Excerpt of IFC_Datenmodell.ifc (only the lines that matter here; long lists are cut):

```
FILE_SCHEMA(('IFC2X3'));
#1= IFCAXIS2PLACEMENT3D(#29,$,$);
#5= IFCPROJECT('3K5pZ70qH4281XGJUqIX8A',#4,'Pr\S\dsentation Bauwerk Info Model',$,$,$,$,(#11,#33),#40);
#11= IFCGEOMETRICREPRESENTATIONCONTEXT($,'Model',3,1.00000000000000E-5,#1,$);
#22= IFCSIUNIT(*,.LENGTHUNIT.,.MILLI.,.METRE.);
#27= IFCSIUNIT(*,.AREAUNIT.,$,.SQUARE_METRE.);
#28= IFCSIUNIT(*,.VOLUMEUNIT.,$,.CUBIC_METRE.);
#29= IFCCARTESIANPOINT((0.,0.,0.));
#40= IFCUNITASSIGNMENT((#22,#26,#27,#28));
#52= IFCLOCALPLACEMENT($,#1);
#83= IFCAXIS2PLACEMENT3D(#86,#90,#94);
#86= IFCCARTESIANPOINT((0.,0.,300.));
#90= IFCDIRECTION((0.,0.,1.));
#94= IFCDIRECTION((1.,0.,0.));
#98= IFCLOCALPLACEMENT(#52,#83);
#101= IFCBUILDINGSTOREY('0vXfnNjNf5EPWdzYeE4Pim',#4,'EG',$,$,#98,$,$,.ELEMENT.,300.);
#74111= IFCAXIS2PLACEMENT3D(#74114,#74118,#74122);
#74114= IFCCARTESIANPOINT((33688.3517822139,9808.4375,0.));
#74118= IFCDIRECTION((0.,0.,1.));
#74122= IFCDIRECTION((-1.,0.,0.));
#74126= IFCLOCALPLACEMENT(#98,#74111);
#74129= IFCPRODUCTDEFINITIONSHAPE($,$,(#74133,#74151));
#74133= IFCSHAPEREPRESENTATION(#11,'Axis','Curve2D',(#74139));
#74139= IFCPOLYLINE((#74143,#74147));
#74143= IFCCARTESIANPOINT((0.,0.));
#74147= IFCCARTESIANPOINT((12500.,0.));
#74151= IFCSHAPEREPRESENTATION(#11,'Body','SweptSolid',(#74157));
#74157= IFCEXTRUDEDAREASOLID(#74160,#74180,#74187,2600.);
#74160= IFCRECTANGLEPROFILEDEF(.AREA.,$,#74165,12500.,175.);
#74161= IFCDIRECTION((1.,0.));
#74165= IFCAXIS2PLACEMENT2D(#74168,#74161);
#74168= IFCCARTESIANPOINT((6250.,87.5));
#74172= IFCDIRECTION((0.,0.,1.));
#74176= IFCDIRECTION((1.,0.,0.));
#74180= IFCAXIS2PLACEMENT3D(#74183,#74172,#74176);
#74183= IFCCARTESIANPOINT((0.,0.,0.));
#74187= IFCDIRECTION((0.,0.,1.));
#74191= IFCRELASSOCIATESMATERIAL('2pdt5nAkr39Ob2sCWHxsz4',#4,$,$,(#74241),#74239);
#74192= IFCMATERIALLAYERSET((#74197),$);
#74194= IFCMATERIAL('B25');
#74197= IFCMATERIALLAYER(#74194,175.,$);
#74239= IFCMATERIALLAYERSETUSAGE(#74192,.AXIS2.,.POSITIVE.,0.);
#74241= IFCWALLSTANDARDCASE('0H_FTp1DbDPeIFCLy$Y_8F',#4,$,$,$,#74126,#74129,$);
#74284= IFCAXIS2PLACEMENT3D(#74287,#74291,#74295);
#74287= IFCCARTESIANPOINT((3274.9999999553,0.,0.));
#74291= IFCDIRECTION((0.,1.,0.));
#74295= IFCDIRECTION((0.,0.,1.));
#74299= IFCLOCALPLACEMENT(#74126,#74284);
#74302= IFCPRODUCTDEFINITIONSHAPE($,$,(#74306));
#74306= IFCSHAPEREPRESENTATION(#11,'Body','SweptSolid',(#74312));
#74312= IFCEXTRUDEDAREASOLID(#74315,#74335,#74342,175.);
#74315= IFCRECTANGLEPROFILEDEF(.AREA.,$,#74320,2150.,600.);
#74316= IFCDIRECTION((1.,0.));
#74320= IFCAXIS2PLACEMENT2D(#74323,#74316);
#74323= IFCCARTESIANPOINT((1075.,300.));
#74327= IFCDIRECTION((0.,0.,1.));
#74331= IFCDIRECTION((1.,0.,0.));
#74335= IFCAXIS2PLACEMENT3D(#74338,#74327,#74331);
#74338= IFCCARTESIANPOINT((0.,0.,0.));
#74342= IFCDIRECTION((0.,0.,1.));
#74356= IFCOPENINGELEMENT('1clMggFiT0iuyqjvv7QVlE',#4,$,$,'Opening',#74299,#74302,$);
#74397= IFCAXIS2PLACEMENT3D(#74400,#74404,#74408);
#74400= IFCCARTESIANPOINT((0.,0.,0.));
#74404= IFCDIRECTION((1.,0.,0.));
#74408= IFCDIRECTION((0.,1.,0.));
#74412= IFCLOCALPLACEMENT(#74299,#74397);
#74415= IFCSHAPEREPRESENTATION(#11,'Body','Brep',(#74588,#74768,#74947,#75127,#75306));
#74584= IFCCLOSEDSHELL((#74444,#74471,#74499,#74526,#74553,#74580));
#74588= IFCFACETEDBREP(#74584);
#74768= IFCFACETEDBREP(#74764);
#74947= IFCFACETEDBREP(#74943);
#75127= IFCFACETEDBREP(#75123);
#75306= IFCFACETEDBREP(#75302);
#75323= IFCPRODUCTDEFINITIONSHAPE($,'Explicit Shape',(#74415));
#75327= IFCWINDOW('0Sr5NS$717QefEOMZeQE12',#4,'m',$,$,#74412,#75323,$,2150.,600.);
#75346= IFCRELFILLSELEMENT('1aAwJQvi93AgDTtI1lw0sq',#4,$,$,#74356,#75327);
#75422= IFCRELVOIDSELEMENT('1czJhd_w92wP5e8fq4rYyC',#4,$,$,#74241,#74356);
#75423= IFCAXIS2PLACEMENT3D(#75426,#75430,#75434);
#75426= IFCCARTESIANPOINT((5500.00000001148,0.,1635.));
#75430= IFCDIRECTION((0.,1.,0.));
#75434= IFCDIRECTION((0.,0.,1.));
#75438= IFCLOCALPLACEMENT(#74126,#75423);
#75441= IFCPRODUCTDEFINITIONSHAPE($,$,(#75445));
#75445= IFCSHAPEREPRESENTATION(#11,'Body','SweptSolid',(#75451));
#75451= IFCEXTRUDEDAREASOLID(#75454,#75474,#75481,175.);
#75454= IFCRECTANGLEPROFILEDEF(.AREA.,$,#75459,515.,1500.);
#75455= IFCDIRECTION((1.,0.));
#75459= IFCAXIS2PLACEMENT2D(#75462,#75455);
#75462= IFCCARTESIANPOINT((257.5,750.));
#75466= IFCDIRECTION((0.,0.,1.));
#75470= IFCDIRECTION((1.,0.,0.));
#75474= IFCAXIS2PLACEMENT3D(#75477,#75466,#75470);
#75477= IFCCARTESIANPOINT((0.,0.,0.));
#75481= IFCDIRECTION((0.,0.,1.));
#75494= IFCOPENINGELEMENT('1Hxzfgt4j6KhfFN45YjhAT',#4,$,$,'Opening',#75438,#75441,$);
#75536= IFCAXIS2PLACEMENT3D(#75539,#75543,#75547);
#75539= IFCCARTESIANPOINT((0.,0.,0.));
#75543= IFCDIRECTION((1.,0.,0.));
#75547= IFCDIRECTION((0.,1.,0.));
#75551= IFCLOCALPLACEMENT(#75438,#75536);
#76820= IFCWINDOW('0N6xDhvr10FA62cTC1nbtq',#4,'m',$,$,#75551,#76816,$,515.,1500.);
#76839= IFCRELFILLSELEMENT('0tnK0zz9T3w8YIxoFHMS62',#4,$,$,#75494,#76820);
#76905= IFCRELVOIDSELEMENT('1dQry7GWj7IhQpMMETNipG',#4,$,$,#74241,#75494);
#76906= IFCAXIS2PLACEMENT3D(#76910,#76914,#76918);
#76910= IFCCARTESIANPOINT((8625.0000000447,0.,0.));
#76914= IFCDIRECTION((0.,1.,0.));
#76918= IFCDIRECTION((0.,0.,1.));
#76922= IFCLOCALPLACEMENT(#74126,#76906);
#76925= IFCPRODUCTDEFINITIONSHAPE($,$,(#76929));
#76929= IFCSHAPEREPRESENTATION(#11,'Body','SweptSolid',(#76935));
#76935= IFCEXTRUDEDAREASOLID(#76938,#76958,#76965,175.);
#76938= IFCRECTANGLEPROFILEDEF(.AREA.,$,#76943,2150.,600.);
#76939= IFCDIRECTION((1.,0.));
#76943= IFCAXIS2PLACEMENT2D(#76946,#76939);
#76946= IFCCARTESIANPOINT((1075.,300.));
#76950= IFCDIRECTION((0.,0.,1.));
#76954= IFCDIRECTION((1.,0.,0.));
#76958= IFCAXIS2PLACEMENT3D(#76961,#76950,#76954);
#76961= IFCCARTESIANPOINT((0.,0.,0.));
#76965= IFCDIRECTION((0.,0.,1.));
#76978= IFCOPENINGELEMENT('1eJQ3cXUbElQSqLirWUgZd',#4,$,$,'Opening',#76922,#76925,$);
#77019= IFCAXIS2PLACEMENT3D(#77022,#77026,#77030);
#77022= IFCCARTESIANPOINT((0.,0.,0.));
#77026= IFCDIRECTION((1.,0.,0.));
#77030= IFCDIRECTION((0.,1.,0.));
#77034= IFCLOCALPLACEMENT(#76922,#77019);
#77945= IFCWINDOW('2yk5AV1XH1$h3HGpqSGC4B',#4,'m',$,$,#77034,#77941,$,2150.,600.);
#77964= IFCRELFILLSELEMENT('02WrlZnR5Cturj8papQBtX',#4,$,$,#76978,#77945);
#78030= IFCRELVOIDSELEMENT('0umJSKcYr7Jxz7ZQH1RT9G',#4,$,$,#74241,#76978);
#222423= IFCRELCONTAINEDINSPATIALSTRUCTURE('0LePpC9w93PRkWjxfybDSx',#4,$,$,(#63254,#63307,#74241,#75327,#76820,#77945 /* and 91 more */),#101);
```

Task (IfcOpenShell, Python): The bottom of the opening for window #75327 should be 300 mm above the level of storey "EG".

```python
import numpy as np
import ifcopenshell
import ifcopenshell.api.geometry
import ifcopenshell.geom
import ifcopenshell.util.element
import ifcopenshell.util.placement
import ifcopenshell.util.shape
import ifcopenshell.util.unit

model = ifcopenshell.open("IFC_Datenmodell.ifc")
unit_scale = ifcopenshell.util.unit.calculate_unit_scale(model)

window = model.by_guid("0Sr5NS$717QefEOMZeQE12")
opening = window.FillsVoids[0].RelatingOpeningElement
storey = ifcopenshell.util.element.get_container(window, ifc_class="IfcBuildingStorey")
level = ifcopenshell.util.placement.get_local_placement(storey.ObjectPlacement)[2, 3]

# The opening's origin need not be at the sill, so measure its lowest point.
shape = ifcopenshell.geom.create_shape(ifcopenshell.geom.settings(), opening)
bottom = ifcopenshell.util.shape.get_shape_bottom_elevation(shape, shape.geometry) / unit_scale
dz = level + 0.3 / unit_scale - bottom

shift = np.array([0.0, 0.0, dz])
# The window is placed relative to its opening, so it follows when the opening moves.
matrix = ifcopenshell.util.placement.get_local_placement(opening.ObjectPlacement)
matrix[:3, 3] += shift
ifcopenshell.api.geometry.edit_object_placement(
    model, product=opening, matrix=matrix, is_si=False, should_transform_children=True
)

print(f"moved by {dz * unit_scale:+.3f} m")

model.write("IFC_Datenmodell_updated.ifc")
```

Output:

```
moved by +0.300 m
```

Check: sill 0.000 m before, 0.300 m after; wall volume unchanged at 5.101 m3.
